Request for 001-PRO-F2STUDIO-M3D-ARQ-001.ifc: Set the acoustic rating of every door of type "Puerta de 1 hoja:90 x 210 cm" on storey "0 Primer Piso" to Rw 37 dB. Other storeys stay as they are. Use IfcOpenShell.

First a look at what the model holds.

```python
import ifcopenshell
import ifcopenshell.util.element

model = ifcopenshell.open("001-PRO-F2STUDIO-M3D-ARQ-001.ifc")
print(model.schema)
storey = next(s for s in model.by_type("IfcBuildingStorey") if s.Name == "0 Primer Piso")
doors = [e for e in ifcopenshell.util.element.get_decomposition(storey) if e.is_a("IfcDoor")]
seen = {}
for e in doors:
    element_type = ifcopenshell.util.element.get_type(e)
    key = (element_type.Name if element_type != e and element_type else None, ifcopenshell.util.element.get_pset(e, "Pset_DoorCommon", "AcousticRating"))
    seen[key] = seen.get(key, 0) + 1
for (name, value), count in sorted(seen.items(), key=str):
    print(count, "x", name, "|", value)
```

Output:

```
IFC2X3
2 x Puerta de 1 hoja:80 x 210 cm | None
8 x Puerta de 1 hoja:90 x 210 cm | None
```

```python
import ifcopenshell
import ifcopenshell.api.pset
import ifcopenshell.util.element

model = ifcopenshell.open("001-PRO-F2STUDIO-M3D-ARQ-001.ifc")

storey = next(s for s in model.by_type("IfcBuildingStorey") if s.Name == "0 Primer Piso")
doors = [e for e in ifcopenshell.util.element.get_decomposition(storey) if e.is_a("IfcDoor")]

count = 0
for e in doors:
    element_type = ifcopenshell.util.element.get_type(e)
    if element_type in (None, e) or element_type.Name != "Puerta de 1 hoja:90 x 210 cm":
        continue
    # add_pset returns the element's existing set when there is one.
    pset = ifcopenshell.api.pset.add_pset(model, product=e, name="Pset_DoorCommon")
    ifcopenshell.api.pset.edit_pset(model, pset=pset, properties={"AcousticRating": "Rw 37 dB"})
    count += 1

print(count, "doors updated")

model.write("001-PRO-F2STUDIO-M3D-ARQ-001_updated.ifc")
```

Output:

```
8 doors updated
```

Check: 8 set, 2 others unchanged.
